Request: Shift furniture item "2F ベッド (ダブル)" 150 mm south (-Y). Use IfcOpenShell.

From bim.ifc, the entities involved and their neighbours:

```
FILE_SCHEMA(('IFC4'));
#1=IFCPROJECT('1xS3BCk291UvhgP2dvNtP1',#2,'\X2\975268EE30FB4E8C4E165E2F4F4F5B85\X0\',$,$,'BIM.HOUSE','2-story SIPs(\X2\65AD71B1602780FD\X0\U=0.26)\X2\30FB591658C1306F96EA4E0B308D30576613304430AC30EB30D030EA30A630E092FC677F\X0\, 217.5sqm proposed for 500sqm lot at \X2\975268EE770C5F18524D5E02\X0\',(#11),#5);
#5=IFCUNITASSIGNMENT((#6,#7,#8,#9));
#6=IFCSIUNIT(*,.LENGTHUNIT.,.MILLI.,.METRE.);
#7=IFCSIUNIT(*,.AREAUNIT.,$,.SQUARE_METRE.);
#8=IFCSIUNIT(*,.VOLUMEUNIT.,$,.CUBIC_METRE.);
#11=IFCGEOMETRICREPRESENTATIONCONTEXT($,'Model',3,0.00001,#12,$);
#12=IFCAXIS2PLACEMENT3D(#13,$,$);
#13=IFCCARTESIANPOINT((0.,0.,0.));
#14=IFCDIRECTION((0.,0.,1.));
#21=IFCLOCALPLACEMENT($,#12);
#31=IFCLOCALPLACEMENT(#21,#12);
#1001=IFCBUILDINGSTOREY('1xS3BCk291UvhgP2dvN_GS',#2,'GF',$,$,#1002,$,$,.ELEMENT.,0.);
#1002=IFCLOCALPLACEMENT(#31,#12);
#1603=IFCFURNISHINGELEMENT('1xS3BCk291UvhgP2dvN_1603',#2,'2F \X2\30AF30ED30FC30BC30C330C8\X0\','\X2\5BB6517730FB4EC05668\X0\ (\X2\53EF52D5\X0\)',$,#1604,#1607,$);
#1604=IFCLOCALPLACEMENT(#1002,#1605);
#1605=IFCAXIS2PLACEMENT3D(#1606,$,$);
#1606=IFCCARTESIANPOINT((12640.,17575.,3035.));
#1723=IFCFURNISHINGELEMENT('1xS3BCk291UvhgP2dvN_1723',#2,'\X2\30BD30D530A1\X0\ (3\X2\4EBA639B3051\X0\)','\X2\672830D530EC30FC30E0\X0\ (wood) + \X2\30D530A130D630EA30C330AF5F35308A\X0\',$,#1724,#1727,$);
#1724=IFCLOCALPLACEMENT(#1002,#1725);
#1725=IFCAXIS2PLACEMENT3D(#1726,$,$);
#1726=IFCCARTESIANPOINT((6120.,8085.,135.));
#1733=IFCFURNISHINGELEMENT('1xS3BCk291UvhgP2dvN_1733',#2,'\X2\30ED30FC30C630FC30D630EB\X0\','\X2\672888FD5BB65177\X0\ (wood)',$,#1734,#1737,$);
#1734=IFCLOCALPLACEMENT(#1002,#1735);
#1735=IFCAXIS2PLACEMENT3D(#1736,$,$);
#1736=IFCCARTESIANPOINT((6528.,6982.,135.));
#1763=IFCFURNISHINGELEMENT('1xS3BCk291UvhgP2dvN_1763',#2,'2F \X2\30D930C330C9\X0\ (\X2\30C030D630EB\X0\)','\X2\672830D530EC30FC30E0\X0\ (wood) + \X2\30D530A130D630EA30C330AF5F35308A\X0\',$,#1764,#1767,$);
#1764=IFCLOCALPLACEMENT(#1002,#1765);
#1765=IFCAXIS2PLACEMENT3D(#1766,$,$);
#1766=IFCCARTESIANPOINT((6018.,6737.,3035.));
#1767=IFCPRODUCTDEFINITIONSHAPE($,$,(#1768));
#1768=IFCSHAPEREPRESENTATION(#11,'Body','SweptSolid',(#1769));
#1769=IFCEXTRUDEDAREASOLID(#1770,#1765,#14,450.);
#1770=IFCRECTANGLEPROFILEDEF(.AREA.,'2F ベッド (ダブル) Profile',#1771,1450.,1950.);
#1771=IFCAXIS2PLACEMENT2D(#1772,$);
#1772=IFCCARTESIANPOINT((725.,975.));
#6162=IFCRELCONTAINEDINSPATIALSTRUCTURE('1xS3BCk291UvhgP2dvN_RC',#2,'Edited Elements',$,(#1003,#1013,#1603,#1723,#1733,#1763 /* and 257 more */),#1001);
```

```python
import ifcopenshell
import ifcopenshell.api.geometry
import ifcopenshell.util.placement

model = ifcopenshell.open("bim.ifc")

item = model.by_guid("1xS3BCk291UvhgP2dvN_1763")
matrix = ifcopenshell.util.placement.get_local_placement(item.ObjectPlacement)
matrix[1, 3] -= 150.0
ifcopenshell.api.geometry.edit_object_placement(model, product=item, matrix=matrix, is_si=False)

print(ifcopenshell.util.placement.get_local_placement(item.ObjectPlacement).round(3) + 0.0)

model.write("bim_v2.ifc")
```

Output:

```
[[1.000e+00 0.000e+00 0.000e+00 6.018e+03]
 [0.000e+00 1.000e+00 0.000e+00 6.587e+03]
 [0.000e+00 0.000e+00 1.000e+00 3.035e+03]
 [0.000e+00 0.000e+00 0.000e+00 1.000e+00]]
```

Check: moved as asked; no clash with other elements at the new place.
